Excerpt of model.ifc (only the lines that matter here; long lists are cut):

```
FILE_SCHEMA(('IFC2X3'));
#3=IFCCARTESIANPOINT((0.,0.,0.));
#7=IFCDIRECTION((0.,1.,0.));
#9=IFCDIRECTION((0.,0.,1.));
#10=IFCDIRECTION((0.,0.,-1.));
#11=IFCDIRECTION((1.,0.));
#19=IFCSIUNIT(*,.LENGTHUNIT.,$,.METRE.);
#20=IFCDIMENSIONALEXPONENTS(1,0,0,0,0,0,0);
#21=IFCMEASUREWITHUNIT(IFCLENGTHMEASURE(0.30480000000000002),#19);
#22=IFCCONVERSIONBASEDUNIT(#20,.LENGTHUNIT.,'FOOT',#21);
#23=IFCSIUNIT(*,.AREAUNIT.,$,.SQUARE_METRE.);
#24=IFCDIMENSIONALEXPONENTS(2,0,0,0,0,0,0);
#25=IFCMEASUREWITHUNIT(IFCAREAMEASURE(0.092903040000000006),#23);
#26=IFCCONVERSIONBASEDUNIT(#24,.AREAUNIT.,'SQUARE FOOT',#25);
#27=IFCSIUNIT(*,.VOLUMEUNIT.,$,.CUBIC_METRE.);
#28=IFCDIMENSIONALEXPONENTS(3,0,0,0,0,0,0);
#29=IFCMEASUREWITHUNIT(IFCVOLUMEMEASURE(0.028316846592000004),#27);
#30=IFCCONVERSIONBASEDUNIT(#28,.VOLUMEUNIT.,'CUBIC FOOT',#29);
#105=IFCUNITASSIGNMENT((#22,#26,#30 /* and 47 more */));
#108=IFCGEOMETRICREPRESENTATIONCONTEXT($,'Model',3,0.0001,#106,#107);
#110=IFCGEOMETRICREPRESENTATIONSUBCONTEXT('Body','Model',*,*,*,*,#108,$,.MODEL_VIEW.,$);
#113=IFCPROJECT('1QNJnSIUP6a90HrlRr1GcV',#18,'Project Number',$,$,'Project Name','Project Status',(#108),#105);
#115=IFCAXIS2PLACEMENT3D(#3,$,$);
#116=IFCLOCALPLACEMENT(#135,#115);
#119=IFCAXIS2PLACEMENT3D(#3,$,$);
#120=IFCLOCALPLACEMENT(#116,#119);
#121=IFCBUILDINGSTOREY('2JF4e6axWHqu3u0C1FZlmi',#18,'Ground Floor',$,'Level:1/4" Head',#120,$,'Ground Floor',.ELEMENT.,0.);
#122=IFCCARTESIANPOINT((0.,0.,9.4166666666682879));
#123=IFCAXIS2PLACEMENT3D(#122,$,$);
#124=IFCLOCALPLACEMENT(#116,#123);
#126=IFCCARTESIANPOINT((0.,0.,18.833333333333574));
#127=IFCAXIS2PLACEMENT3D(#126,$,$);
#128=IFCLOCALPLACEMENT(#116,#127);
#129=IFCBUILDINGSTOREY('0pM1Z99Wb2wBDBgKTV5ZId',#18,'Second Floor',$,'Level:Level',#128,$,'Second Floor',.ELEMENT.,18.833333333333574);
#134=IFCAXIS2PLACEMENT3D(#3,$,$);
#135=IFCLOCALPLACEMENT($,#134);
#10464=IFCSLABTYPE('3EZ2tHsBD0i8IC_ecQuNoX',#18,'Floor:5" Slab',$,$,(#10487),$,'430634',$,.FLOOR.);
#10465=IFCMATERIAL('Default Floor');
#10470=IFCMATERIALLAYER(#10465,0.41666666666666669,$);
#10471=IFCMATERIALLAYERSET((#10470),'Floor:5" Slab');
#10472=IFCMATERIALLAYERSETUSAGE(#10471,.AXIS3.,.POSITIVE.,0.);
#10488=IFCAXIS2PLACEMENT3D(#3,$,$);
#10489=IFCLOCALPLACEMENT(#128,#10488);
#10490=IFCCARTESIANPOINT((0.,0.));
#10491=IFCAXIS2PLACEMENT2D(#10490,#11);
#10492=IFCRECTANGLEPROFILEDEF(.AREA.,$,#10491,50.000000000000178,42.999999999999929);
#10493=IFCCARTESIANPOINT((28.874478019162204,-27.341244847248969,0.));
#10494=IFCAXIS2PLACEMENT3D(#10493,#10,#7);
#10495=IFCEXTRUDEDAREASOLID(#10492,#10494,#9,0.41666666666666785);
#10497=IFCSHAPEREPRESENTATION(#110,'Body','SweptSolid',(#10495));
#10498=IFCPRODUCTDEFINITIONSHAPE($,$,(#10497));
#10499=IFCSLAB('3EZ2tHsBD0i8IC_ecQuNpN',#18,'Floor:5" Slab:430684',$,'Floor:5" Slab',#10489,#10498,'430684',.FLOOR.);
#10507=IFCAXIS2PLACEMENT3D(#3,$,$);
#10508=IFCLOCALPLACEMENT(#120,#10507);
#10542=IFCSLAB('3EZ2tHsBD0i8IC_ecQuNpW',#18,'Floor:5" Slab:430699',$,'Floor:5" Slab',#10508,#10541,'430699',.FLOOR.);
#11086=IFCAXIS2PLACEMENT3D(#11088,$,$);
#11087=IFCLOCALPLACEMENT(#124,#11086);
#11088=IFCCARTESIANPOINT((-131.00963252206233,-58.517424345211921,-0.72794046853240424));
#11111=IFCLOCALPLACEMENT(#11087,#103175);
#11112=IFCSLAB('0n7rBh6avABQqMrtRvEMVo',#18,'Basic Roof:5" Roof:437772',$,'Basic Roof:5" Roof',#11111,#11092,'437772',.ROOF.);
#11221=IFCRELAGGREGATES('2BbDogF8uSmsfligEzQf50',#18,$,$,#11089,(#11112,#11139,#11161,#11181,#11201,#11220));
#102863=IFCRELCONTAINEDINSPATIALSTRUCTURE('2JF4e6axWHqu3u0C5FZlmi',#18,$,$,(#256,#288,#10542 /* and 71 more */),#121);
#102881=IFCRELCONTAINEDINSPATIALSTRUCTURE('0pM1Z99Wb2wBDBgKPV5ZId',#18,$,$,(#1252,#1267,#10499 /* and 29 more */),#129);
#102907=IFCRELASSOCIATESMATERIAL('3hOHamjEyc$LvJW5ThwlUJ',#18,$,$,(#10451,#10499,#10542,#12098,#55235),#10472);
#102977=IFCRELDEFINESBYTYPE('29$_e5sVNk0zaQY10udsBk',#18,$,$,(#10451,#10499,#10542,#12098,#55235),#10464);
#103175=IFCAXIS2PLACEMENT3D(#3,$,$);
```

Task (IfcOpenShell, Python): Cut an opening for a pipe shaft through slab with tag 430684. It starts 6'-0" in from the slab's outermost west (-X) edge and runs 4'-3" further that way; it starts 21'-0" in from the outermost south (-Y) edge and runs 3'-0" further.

```python
import numpy as np
import ifcopenshell
import ifcopenshell.api.feature
import ifcopenshell.api.geometry
import ifcopenshell.api.root
import ifcopenshell.geom
import ifcopenshell.util.placement
import ifcopenshell.util.representation
import ifcopenshell.util.shape
import ifcopenshell.util.unit

model = ifcopenshell.open("model.ifc")
unit_scale = ifcopenshell.util.unit.calculate_unit_scale(model)
settings = ifcopenshell.geom.settings()


def volume(element):
    """Net volume in cubic metres, openings subtracted."""
    shape = ifcopenshell.geom.create_shape(settings, element)
    return ifcopenshell.util.shape.get_volume(shape.geometry)


slab = model.by_guid("3EZ2tHsBD0i8IC_ecQuNpN")
before = volume(slab)

# Extent in the slab's own axes, in metres. The edges named are its -X and -Y sides.
slab_shape = ifcopenshell.geom.create_shape(settings, slab)
vertices = ifcopenshell.util.shape.get_vertices(slab_shape.geometry)
x_min, y_min, bottom = vertices.min(axis=0)
top = vertices[:, 2].max()

opening = ifcopenshell.api.root.create_entity(model, ifc_class="IfcOpeningElement", name="Pipe shaft opening")
context = ifcopenshell.util.representation.get_context(model, "Model", "Body", "MODEL_VIEW")
width, depth = 1.2954, 0.9144
outline = [(0.0, 0.0), (width, 0.0), (width, depth), (0.0, depth), (0.0, 0.0)]
# Overshoot both faces by 50 mm so the cut is clean.
shape = ifcopenshell.api.geometry.add_slab_representation(
    model, context=context, depth=top - bottom + 0.1, polyline=outline
)
ifcopenshell.api.geometry.assign_representation(model, product=opening, representation=shape)

matrix = ifcopenshell.util.placement.get_local_placement(slab.ObjectPlacement)
matrix[:, 3] = matrix @ np.append(np.array([x_min + 1.8288, y_min + 6.4008, bottom - 0.05]) / unit_scale, 1.0)
ifcopenshell.api.geometry.edit_object_placement(model, product=opening, matrix=matrix, is_si=False)
ifcopenshell.api.feature.add_feature(model, feature=opening, element=slab)

after = volume(slab)

print(f"slab volume {before:.3f} -> {after:.3f} m3")

model.write("model_updated.ifc")
```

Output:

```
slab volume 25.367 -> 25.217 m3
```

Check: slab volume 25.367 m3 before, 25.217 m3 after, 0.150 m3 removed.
